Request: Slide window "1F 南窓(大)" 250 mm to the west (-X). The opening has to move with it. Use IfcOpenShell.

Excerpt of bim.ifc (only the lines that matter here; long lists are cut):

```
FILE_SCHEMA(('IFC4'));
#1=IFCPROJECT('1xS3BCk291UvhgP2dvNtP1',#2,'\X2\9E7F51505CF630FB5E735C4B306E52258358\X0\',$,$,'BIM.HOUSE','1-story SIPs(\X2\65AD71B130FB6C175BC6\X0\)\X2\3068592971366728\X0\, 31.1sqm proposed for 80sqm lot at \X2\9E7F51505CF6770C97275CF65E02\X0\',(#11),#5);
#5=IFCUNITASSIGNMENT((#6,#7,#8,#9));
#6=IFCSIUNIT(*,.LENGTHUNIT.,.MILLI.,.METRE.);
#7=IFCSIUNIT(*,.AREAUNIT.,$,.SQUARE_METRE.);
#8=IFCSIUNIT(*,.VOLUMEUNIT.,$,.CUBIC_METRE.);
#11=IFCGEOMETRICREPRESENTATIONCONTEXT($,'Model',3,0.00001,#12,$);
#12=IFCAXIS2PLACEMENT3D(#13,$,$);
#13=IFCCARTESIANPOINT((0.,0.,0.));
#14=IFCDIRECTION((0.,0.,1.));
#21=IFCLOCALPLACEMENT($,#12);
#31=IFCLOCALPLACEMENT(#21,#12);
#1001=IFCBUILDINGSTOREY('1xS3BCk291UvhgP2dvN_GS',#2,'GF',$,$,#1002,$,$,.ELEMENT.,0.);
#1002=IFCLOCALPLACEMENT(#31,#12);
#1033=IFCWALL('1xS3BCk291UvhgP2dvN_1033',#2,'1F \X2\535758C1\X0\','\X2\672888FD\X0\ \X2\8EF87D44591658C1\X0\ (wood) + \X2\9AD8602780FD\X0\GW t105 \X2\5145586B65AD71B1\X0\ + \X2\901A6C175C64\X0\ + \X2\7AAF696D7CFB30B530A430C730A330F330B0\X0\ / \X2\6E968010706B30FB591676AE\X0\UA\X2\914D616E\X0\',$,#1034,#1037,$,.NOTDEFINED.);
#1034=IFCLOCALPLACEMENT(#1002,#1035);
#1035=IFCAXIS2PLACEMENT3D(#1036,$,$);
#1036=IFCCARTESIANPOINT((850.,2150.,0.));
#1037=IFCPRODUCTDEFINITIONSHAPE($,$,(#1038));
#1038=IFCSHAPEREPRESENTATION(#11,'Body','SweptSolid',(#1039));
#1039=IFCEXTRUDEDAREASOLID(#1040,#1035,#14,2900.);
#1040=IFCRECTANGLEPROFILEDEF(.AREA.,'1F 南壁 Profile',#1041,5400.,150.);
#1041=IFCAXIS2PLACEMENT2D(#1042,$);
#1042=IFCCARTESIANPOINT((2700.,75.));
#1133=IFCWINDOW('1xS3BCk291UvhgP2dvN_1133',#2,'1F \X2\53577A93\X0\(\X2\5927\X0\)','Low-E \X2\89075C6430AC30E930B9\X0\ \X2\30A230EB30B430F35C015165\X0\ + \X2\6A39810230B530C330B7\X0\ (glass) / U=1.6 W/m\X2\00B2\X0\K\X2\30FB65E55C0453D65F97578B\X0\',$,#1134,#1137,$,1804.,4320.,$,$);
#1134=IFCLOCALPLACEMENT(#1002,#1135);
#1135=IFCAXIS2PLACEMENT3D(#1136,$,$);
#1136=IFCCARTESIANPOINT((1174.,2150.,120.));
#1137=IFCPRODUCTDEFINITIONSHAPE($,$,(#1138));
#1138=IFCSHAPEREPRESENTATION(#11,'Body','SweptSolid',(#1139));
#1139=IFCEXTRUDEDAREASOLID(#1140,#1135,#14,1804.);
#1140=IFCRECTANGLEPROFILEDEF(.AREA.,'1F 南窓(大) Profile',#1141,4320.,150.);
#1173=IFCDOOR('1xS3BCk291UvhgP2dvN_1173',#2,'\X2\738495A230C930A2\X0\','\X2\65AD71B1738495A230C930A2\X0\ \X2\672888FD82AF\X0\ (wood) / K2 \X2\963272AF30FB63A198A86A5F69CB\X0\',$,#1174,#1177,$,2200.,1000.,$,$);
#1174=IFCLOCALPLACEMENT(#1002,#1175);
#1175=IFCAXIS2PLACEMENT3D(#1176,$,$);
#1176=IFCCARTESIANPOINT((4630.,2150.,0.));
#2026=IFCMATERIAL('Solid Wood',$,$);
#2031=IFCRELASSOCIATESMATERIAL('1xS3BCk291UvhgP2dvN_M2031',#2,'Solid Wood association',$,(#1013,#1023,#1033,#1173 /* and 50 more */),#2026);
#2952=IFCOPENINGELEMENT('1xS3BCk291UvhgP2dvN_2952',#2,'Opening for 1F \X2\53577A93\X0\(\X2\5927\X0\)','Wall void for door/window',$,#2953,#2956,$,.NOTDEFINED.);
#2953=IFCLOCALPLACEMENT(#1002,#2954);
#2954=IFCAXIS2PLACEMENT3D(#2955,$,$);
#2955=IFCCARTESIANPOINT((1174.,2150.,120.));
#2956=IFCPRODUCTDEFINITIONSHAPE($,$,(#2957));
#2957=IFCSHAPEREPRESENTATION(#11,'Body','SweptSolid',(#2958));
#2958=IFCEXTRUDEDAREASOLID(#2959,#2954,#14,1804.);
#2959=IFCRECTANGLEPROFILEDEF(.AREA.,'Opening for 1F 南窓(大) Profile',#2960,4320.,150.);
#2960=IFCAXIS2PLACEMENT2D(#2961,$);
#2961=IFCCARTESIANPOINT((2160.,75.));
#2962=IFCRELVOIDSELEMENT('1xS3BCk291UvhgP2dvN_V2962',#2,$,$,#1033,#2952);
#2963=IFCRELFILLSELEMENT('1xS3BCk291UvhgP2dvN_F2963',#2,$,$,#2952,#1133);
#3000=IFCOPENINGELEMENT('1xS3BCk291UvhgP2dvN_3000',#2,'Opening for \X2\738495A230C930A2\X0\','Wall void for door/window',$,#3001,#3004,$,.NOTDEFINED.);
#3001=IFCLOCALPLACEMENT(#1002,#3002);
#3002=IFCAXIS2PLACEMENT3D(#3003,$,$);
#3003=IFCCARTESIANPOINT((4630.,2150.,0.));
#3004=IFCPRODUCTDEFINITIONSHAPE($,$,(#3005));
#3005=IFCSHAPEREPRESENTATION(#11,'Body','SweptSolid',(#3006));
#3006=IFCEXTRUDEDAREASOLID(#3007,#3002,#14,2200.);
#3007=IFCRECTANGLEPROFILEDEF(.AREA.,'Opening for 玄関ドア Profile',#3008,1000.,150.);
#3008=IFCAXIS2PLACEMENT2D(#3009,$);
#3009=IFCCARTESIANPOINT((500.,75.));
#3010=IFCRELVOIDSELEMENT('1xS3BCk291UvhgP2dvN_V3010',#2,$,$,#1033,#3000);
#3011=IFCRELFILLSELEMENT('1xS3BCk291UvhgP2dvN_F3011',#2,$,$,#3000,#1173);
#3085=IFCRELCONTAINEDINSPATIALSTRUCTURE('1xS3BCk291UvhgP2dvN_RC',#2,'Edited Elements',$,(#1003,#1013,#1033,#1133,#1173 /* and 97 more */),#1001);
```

```python
import ifcopenshell
import ifcopenshell.api.geometry
import ifcopenshell.util.placement
import ifcopenshell.util.unit

model = ifcopenshell.open("bim.ifc")
unit_scale = ifcopenshell.util.unit.calculate_unit_scale(model)

window = model.by_guid("1xS3BCk291UvhgP2dvN_1133")
opening = window.FillsVoids[0].RelatingOpeningElement
wall = opening.VoidsElements[0].RelatingBuildingElement

wall_matrix = ifcopenshell.util.placement.get_local_placement(wall.ObjectPlacement)
shift = wall_matrix[:3, 0] * -0.25 / unit_scale
before = ifcopenshell.util.placement.get_local_placement(window.ObjectPlacement)[:3, 3].copy()

# The window is not placed relative to its opening, so move both.
for product in (opening, window):
    matrix = ifcopenshell.util.placement.get_local_placement(product.ObjectPlacement)
    matrix[:3, 3] += shift
    ifcopenshell.api.geometry.edit_object_placement(model, product=product, matrix=matrix, is_si=False)

after = ifcopenshell.util.placement.get_local_placement(window.ObjectPlacement)[:3, 3]
print("window moved by", (after - before).round(3) + 0.0)

model.write("bim_v2.ifc")
```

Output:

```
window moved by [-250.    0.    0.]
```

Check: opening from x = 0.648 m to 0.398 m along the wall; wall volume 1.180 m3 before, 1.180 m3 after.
